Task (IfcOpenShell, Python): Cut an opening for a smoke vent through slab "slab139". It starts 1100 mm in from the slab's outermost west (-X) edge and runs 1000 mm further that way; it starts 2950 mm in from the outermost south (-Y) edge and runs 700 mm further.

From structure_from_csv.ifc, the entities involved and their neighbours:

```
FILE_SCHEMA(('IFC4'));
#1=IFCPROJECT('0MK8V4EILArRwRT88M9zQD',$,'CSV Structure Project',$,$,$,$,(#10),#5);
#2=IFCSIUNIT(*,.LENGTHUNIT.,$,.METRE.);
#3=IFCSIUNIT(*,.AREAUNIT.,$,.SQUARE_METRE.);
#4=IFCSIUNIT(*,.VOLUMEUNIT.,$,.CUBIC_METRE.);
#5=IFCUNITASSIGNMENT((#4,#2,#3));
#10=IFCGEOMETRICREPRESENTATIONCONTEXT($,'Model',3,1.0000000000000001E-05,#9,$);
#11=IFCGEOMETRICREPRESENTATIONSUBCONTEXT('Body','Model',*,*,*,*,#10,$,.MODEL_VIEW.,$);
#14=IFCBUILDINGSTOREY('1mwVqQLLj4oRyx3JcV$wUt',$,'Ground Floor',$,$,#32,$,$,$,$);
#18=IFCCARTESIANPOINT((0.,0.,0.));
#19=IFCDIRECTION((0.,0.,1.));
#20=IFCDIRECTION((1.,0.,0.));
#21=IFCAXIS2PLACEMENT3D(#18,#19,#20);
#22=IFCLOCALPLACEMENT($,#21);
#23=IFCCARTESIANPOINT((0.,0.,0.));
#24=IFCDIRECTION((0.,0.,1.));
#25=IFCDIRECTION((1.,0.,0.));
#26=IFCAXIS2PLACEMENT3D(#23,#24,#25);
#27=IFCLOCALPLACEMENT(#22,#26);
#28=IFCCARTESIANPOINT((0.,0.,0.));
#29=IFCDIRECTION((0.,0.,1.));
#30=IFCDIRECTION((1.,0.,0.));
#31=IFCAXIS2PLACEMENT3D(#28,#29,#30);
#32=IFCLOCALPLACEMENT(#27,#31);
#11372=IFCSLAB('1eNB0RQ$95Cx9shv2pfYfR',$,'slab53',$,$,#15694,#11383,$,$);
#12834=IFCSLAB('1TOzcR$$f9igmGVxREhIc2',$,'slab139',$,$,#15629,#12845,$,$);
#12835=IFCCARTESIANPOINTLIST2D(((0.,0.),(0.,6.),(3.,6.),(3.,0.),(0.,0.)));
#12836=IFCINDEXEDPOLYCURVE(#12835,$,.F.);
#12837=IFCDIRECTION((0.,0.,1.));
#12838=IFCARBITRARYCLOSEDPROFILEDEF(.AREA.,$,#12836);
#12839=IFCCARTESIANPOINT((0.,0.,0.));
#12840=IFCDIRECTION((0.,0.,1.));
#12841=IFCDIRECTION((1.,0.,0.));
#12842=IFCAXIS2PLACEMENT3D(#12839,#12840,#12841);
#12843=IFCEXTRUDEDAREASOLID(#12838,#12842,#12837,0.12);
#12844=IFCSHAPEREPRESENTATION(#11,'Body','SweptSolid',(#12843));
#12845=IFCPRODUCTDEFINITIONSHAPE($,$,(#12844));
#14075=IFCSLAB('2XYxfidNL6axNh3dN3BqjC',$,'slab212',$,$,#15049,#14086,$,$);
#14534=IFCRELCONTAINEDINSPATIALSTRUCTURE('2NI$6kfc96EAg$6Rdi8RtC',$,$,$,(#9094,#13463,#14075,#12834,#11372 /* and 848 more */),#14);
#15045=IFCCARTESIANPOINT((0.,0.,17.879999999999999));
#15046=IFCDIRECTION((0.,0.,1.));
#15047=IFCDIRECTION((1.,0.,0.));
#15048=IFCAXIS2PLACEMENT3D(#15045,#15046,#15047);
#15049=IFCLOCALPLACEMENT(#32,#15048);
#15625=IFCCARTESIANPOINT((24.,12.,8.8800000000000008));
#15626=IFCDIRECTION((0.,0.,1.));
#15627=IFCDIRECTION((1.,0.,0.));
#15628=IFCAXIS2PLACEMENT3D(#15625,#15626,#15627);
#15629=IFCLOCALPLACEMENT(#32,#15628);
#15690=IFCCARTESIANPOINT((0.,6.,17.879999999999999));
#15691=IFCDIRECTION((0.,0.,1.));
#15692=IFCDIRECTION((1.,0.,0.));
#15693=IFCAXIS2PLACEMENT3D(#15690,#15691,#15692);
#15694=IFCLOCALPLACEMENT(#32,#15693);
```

```python
import numpy as np
import ifcopenshell
import ifcopenshell.api.feature
import ifcopenshell.api.geometry
import ifcopenshell.api.root
import ifcopenshell.geom
import ifcopenshell.util.placement
import ifcopenshell.util.representation
import ifcopenshell.util.shape
import ifcopenshell.util.unit

model = ifcopenshell.open("structure_from_csv.ifc")
unit_scale = ifcopenshell.util.unit.calculate_unit_scale(model)
settings = ifcopenshell.geom.settings()


def volume(element):
    """Net volume in cubic metres, openings subtracted."""
    shape = ifcopenshell.geom.create_shape(settings, element)
    return ifcopenshell.util.shape.get_volume(shape.geometry)


slab = model.by_guid("1TOzcR$$f9igmGVxREhIc2")
before = volume(slab)

# Extent in the slab's own axes, in metres. The edges named are its -X and -Y sides.
slab_shape = ifcopenshell.geom.create_shape(settings, slab)
vertices = ifcopenshell.util.shape.get_vertices(slab_shape.geometry)
x_min, y_min, bottom = vertices.min(axis=0)
top = vertices[:, 2].max()

opening = ifcopenshell.api.root.create_entity(model, ifc_class="IfcOpeningElement", name="Smoke vent opening", predefined_type="OPENING")
context = ifcopenshell.util.representation.get_context(model, "Model", "Body", "MODEL_VIEW")
width, depth = 1, 0.7
outline = [(0.0, 0.0), (width, 0.0), (width, depth), (0.0, depth), (0.0, 0.0)]
# Overshoot both faces by 50 mm so the cut is clean.
shape = ifcopenshell.api.geometry.add_slab_representation(
    model, context=context, depth=top - bottom + 0.1, polyline=outline
)
ifcopenshell.api.geometry.assign_representation(model, product=opening, representation=shape)

matrix = ifcopenshell.util.placement.get_local_placement(slab.ObjectPlacement)
matrix[:, 3] = matrix @ np.append(np.array([x_min + 1.1, y_min + 2.95, bottom - 0.05]) / unit_scale, 1.0)
ifcopenshell.api.geometry.edit_object_placement(model, product=opening, matrix=matrix, is_si=False)
ifcopenshell.api.feature.add_feature(model, feature=opening, element=slab)

after = volume(slab)

print(f"slab volume {before:.3f} -> {after:.3f} m3")

model.write("structure_from_csv-out.ifc")
```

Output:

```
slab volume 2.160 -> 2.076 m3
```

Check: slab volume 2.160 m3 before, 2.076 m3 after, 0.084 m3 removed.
